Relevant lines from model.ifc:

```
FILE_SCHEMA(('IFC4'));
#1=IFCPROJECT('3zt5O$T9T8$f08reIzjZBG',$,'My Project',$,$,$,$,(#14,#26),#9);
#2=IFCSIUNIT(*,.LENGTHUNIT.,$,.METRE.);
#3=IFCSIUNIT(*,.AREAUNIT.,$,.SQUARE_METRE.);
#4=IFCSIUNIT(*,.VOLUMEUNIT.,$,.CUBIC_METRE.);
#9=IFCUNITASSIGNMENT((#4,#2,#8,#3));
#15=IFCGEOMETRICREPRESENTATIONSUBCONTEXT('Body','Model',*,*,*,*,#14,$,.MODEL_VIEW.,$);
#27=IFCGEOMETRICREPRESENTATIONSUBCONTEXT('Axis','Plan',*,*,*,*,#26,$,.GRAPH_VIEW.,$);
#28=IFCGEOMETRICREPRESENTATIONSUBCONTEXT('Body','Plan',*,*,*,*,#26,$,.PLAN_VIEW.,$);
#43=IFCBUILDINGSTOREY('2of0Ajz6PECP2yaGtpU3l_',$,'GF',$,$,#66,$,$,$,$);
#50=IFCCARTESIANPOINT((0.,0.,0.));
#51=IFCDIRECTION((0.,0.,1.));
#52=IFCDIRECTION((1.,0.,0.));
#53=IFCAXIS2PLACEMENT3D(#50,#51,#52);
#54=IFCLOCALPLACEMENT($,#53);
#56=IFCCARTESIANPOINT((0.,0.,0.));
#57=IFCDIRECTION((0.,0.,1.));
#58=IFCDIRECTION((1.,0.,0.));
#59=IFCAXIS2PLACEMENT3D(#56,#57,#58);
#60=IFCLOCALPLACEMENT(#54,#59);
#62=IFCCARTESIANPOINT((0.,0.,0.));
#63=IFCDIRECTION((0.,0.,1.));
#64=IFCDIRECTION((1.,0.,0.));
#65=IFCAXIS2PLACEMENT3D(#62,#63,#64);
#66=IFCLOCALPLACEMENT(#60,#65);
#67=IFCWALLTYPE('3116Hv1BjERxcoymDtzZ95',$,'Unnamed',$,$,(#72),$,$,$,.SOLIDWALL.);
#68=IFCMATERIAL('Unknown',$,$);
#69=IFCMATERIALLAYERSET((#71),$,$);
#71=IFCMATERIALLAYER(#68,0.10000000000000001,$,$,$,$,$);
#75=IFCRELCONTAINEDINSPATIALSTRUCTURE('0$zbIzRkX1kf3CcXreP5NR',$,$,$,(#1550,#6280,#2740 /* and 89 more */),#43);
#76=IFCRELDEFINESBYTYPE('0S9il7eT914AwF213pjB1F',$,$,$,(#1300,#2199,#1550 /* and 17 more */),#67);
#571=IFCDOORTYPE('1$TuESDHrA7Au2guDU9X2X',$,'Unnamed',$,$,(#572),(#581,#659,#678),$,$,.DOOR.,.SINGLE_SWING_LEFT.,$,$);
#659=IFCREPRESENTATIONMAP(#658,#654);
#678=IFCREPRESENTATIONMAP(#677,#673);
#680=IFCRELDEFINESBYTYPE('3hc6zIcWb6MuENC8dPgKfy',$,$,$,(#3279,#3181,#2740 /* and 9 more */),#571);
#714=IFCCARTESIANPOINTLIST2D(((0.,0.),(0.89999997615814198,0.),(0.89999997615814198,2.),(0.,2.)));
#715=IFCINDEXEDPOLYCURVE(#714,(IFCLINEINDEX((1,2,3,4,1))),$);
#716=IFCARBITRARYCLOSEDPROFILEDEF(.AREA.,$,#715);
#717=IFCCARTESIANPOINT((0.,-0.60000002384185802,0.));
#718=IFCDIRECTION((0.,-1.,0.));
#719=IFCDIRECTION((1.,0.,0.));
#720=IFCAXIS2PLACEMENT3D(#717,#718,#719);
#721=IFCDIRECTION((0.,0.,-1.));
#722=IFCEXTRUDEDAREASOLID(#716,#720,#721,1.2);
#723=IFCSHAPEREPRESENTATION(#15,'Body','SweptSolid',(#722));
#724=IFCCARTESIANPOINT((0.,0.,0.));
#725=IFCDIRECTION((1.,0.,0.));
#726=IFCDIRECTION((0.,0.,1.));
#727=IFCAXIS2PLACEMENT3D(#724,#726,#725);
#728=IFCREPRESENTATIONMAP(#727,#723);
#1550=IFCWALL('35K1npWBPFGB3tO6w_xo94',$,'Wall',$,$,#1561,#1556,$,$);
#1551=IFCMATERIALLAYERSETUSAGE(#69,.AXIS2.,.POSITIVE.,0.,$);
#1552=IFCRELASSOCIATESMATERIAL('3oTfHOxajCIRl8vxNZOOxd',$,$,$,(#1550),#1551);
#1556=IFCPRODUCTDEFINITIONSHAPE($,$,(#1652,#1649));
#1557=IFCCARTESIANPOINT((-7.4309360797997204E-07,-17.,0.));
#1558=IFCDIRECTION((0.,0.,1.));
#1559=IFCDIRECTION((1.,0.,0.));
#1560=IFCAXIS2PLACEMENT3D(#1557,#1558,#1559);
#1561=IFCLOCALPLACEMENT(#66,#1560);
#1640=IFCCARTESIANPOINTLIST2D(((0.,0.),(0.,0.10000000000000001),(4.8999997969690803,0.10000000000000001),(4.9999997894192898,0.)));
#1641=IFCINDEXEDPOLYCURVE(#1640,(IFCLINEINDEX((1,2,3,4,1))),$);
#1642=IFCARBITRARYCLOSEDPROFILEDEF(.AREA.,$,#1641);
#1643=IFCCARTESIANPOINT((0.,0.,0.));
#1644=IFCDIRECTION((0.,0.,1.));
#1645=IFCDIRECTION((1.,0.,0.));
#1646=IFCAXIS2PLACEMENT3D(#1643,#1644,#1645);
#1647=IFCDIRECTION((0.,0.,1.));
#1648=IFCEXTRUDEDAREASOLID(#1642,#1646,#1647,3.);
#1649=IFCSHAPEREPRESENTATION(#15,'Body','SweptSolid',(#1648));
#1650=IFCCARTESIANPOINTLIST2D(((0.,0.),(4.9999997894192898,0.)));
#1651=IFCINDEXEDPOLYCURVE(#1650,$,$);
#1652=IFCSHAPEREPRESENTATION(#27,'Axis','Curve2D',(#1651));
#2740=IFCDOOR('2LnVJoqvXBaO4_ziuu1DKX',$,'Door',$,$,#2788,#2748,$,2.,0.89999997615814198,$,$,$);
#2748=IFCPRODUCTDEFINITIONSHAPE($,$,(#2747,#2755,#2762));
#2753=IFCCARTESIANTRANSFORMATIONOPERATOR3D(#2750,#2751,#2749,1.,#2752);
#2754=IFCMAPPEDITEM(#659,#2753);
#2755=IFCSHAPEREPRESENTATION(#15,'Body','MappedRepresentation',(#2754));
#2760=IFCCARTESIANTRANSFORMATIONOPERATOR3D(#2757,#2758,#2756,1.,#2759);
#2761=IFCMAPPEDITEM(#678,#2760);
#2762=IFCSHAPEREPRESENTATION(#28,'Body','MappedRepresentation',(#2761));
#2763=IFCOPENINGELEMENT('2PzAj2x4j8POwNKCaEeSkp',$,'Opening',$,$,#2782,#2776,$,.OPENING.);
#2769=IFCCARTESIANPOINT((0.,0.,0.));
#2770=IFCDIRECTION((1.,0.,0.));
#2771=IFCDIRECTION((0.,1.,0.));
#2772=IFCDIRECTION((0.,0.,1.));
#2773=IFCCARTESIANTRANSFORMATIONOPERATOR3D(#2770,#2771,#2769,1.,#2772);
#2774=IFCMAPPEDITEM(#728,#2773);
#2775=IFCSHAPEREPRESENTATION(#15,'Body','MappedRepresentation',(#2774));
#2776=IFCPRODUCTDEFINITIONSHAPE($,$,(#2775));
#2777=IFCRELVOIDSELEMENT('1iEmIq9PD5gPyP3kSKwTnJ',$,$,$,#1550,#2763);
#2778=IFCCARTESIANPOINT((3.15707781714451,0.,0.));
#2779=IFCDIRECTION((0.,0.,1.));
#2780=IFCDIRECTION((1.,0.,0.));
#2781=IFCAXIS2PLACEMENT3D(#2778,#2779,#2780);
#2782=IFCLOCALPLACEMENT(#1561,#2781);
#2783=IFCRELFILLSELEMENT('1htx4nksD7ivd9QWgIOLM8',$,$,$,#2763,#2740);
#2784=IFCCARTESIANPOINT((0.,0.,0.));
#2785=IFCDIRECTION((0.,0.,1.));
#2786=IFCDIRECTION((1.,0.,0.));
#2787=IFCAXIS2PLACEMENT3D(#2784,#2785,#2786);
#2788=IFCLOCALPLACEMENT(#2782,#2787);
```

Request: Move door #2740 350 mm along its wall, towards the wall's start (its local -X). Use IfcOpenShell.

```python
import ifcopenshell
import ifcopenshell.api.geometry
import ifcopenshell.util.placement
import ifcopenshell.util.unit

model = ifcopenshell.open("model.ifc")
unit_scale = ifcopenshell.util.unit.calculate_unit_scale(model)

door = model.by_id(2740)
opening = door.FillsVoids[0].RelatingOpeningElement
wall = opening.VoidsElements[0].RelatingBuildingElement

wall_matrix = ifcopenshell.util.placement.get_local_placement(wall.ObjectPlacement)
shift = wall_matrix[:3, 0] * -0.35 / unit_scale
before = ifcopenshell.util.placement.get_local_placement(door.ObjectPlacement)[:3, 3].copy()

# The door is placed relative to its opening, so it follows when the opening moves.
matrix = ifcopenshell.util.placement.get_local_placement(opening.ObjectPlacement)
matrix[:3, 3] += shift
ifcopenshell.api.geometry.edit_object_placement(
    model, product=opening, matrix=matrix, is_si=False, should_transform_children=True
)

after = ifcopenshell.util.placement.get_local_placement(door.ObjectPlacement)[:3, 3]
print("door moved by", (after - before).round(3) + 0.0)

model.write("model_edited.ifc")
```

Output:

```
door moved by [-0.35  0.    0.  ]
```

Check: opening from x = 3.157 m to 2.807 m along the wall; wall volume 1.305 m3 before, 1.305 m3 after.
